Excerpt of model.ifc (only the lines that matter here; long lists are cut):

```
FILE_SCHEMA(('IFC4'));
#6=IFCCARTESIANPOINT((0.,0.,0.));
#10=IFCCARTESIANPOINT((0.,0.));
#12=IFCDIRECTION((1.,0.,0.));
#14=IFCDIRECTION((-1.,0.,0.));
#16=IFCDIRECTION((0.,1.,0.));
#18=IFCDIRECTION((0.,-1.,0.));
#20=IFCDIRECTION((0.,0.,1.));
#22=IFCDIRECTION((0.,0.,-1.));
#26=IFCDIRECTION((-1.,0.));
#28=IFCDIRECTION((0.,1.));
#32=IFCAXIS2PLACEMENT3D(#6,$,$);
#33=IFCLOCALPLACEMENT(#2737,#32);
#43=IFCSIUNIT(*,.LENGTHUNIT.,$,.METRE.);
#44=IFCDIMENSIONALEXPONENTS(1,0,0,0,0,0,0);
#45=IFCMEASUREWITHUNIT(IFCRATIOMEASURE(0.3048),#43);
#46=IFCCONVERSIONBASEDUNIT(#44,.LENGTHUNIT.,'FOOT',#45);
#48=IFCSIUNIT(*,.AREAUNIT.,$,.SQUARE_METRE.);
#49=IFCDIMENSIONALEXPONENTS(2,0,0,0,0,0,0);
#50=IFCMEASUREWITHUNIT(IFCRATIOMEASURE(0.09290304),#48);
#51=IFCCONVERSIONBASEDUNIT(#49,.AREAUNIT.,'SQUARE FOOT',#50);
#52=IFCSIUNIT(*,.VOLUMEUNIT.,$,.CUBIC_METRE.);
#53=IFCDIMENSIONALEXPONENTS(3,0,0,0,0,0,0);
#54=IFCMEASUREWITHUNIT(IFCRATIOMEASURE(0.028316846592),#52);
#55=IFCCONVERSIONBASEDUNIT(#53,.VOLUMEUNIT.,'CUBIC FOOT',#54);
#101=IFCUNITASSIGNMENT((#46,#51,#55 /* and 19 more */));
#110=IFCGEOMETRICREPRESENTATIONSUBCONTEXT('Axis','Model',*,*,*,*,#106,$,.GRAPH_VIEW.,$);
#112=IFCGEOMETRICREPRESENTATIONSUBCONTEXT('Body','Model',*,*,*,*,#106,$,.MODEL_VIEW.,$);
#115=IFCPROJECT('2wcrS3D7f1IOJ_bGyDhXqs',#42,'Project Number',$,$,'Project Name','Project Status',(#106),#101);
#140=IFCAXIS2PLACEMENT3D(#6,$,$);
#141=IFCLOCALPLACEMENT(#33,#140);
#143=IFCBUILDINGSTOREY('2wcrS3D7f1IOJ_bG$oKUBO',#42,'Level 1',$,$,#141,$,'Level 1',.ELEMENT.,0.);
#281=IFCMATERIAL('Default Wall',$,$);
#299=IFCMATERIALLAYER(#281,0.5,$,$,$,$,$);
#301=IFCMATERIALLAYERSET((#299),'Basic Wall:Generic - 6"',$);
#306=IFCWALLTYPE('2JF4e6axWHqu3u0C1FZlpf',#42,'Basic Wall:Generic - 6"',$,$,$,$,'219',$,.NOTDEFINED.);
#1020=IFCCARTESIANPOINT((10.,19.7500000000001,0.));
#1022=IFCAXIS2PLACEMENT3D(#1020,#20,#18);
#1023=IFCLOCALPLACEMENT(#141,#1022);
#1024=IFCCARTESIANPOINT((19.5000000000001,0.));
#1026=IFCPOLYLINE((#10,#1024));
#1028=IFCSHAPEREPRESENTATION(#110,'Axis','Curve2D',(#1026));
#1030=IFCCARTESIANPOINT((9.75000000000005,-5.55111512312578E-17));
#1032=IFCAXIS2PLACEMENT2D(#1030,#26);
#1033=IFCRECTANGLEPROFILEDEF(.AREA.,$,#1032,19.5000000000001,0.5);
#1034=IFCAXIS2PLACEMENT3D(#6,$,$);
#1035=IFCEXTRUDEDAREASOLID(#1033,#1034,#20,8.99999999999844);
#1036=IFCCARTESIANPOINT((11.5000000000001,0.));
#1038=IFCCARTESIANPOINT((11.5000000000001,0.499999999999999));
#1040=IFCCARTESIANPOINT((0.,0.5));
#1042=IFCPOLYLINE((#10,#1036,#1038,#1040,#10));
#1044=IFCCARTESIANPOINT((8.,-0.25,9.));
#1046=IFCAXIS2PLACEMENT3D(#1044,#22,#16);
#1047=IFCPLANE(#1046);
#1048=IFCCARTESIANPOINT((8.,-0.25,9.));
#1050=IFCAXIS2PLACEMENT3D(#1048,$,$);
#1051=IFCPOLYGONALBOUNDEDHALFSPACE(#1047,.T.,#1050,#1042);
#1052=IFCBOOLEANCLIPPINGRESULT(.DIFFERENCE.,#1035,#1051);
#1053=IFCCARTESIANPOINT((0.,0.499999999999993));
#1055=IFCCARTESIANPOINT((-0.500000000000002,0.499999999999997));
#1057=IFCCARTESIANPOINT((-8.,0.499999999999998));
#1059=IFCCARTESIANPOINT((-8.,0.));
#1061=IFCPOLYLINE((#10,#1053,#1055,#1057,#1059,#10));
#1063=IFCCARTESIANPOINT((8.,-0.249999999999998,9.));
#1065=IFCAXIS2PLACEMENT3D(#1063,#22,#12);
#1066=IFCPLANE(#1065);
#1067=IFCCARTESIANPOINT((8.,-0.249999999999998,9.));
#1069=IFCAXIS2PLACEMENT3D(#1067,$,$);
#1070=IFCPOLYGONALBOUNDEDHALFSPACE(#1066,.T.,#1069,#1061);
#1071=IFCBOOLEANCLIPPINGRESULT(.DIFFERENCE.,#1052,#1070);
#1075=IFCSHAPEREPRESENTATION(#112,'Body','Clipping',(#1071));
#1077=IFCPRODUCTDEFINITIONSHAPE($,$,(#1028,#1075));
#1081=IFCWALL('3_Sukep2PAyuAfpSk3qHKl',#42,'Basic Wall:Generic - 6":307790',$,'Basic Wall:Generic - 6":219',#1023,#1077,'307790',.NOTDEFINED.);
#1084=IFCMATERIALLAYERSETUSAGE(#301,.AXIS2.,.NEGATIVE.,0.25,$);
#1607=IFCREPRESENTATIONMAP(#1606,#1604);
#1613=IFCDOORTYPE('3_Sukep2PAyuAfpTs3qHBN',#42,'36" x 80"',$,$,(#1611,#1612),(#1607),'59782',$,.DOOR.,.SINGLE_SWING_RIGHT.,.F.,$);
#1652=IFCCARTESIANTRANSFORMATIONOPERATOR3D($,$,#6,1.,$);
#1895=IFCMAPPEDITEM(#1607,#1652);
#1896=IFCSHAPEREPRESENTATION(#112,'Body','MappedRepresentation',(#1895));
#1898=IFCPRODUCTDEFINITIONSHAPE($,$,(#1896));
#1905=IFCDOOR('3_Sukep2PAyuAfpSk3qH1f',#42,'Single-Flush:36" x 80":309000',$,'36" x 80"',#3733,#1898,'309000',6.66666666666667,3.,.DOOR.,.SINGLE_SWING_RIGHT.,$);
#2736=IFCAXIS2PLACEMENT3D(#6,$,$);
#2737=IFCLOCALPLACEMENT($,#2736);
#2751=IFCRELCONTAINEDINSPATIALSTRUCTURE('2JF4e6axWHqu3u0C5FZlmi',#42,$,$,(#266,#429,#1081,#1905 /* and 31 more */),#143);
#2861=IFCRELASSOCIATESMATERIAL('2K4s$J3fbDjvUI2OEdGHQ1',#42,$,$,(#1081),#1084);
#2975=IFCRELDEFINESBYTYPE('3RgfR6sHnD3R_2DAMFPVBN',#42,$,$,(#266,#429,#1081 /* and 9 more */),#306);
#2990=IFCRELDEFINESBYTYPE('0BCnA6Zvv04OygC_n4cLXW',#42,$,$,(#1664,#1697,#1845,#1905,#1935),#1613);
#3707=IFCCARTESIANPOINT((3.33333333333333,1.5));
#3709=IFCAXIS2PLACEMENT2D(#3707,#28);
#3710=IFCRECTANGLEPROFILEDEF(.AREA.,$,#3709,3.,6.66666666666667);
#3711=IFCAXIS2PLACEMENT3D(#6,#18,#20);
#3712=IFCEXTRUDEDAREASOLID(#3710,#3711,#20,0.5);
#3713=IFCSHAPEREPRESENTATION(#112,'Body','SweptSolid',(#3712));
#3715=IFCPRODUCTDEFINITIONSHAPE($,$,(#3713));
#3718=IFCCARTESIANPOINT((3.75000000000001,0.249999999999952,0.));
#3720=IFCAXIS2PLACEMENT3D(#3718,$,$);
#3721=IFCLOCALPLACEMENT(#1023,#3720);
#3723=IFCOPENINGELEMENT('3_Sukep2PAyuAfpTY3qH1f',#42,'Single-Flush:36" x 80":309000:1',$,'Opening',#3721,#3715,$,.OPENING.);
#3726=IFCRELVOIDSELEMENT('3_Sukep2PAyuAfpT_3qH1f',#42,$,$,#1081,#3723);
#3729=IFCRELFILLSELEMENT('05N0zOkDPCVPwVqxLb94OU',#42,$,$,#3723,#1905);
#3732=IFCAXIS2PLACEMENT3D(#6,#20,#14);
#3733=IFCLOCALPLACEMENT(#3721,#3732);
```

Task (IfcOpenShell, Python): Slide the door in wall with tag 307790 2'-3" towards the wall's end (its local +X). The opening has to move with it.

```python
import ifcopenshell
import ifcopenshell.api.geometry
import ifcopenshell.util.placement
import ifcopenshell.util.unit

model = ifcopenshell.open("model.ifc")
unit_scale = ifcopenshell.util.unit.calculate_unit_scale(model)

door = model.by_guid("3_Sukep2PAyuAfpSk3qH1f")
opening = door.FillsVoids[0].RelatingOpeningElement
wall = opening.VoidsElements[0].RelatingBuildingElement

wall_matrix = ifcopenshell.util.placement.get_local_placement(wall.ObjectPlacement)
shift = wall_matrix[:3, 0] * 27 * 0.0254 / unit_scale
before = ifcopenshell.util.placement.get_local_placement(door.ObjectPlacement)[:3, 3].copy()

# The door is placed relative to its opening, so it follows when the opening moves.
matrix = ifcopenshell.util.placement.get_local_placement(opening.ObjectPlacement)
matrix[:3, 3] += shift
ifcopenshell.api.geometry.edit_object_placement(
    model, product=opening, matrix=matrix, is_si=False, should_transform_children=True
)

after = ifcopenshell.util.placement.get_local_placement(door.ObjectPlacement)[:3, 3]
print("door moved by", (after - before).round(3) + 0.0)

model.write("model_updated.ifc")
```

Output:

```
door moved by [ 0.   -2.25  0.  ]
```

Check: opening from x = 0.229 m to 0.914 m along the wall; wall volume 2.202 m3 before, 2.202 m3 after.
